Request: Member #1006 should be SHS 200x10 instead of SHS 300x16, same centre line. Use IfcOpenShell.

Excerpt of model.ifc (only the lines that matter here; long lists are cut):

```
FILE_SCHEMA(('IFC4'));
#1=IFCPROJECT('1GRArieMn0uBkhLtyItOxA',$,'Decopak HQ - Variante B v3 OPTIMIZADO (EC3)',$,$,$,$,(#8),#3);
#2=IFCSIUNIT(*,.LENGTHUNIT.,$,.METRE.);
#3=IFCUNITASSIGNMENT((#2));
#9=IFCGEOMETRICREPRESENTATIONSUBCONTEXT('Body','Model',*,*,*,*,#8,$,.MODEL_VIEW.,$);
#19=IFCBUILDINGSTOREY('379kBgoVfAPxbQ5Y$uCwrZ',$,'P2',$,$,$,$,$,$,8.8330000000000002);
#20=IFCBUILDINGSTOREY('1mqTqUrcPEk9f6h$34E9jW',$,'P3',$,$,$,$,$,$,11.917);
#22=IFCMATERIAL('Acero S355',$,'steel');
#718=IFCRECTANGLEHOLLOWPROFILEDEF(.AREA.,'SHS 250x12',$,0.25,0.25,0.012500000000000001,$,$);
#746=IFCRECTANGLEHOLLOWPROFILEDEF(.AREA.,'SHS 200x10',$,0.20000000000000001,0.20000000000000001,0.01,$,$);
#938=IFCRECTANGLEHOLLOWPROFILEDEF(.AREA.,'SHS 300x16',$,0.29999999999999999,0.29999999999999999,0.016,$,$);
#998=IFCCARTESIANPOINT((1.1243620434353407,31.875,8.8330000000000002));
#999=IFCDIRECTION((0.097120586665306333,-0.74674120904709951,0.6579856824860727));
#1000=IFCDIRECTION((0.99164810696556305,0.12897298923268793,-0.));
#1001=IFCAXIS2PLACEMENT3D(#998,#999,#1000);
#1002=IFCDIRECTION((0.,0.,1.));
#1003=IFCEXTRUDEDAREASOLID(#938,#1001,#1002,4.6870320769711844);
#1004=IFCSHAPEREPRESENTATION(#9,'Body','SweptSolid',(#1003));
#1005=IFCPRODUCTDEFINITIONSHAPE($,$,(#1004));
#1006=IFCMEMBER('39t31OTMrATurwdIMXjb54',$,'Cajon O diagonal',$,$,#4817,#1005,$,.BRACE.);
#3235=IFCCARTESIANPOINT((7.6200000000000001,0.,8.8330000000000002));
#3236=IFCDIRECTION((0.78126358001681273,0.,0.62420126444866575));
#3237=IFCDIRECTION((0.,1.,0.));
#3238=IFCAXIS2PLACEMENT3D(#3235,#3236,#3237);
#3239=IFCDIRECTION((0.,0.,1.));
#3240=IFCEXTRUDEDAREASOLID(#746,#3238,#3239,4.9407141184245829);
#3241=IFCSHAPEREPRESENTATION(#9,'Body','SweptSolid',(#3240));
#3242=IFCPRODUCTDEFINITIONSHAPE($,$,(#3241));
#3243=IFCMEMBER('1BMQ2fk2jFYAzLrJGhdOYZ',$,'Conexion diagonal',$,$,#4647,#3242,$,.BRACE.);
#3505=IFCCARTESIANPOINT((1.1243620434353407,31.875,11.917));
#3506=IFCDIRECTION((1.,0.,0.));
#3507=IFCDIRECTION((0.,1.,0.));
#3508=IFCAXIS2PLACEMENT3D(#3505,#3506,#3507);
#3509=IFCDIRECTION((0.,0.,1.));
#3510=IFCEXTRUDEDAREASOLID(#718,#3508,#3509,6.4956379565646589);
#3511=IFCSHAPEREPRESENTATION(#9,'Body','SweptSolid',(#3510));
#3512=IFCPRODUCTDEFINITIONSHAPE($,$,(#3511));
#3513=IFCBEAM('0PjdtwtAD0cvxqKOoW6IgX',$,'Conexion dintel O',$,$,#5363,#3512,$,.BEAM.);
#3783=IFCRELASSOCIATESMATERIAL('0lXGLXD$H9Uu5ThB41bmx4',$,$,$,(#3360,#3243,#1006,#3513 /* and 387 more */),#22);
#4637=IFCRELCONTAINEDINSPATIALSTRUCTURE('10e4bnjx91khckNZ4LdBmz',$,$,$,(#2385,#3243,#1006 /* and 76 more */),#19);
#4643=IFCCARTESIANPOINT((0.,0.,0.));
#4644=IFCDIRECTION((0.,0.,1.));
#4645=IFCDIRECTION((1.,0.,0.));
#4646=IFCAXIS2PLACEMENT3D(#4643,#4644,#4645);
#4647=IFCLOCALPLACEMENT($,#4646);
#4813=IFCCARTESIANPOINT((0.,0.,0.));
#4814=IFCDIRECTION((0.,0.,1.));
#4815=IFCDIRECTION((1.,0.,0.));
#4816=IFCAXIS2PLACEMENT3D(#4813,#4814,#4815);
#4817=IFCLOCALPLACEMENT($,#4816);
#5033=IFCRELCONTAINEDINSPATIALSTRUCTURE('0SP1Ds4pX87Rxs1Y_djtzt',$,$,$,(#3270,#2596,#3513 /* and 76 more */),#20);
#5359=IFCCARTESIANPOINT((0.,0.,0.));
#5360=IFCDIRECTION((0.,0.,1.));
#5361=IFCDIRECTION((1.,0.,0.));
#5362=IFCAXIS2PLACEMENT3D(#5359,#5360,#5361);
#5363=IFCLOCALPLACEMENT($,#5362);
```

```python
import ifcopenshell
import ifcopenshell.util.element
import ifcopenshell.util.representation

model = ifcopenshell.open("model.ifc")

member = model.by_id(1006)
source = next(p for p in model.by_type("IfcRectangleHollowProfileDef") if p.ProfileName == "SHS 200x10")

body = ifcopenshell.util.representation.get_representation(member, "Model", "Body")
solid = body.Items[0]
old_profile = solid.SweptArea

# Copy the section's sizes but keep this member's own profile position.
profile = ifcopenshell.util.element.copy(model, source)
profile.Position = old_profile.Position
solid.SweptArea = profile
if not model.get_total_inverses(old_profile):
    ifcopenshell.util.element.remove_deep2(model, old_profile)

print(solid.SweptArea)

model.write("model_rev.ifc")
```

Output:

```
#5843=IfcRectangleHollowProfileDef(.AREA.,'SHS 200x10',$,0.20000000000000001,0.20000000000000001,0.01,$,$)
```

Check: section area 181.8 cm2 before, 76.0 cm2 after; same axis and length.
